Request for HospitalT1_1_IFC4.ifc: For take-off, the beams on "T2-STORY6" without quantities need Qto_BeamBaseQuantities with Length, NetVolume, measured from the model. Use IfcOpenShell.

First a look at what the model holds.

```python
import ifcopenshell
import ifcopenshell.util.element
import ifcopenshell.util.unit

model = ifcopenshell.open("HospitalT1_1_IFC4.ifc")
print(model.schema)
for unit_type in ("LENGTHUNIT", "AREAUNIT", "VOLUMEUNIT"):
    print(unit_type, ifcopenshell.util.unit.calculate_unit_scale(model, unit_type))
storey = next(s for s in model.by_type("IfcBuildingStorey") if s.Name == "T2-STORY6")
beams = [e for e in ifcopenshell.util.element.get_decomposition(storey) if e.is_a("IfcBeam")]
for e in sorted(beams, key=lambda e: e.id()):
    print(e.id(), e.is_a(), e.Name, list(ifcopenshell.util.element.get_psets(e, qtos_only=True)), sep=" | ")
```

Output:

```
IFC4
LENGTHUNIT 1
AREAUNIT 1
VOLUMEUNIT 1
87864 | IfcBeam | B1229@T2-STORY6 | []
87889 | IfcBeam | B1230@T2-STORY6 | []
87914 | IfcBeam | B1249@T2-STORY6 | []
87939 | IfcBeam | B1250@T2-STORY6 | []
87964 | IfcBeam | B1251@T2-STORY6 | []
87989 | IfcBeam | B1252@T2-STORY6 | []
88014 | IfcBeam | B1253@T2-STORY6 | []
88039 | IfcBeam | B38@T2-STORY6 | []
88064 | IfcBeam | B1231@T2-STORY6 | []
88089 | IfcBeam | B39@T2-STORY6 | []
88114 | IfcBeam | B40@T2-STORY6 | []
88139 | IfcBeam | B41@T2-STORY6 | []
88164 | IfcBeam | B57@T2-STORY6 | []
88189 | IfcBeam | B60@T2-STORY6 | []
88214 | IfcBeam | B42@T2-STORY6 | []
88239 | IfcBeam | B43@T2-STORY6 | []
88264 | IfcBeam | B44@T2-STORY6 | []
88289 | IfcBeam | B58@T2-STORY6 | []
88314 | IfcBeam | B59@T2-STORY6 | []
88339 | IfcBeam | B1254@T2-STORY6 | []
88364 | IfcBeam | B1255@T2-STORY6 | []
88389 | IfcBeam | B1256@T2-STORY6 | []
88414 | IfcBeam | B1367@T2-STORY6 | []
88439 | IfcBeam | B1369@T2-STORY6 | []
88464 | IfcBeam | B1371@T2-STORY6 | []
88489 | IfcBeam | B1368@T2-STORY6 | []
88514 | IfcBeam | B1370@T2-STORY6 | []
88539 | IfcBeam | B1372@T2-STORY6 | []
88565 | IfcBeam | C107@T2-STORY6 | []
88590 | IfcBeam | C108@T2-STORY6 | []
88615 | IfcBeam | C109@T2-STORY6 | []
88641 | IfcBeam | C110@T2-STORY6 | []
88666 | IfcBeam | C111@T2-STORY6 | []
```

```python
import ifcopenshell
import ifcopenshell.api.pset
import ifcopenshell.geom
import ifcopenshell.util.element
import ifcopenshell.util.shape
import ifcopenshell.util.unit

model = ifcopenshell.open("HospitalT1_1_IFC4.ifc")
unit_scale = ifcopenshell.util.unit.calculate_unit_scale(model)
volume_scale = ifcopenshell.util.unit.calculate_unit_scale(model, "VOLUMEUNIT")
settings = ifcopenshell.geom.settings()

storey = next(s for s in model.by_type("IfcBuildingStorey") if s.Name == "T2-STORY6")
beams = [e for e in ifcopenshell.util.element.get_decomposition(storey) if e.is_a("IfcBeam")]

for e in sorted(beams, key=lambda e: e.id()):
    if ifcopenshell.util.element.get_psets(e, qtos_only=True, should_inherit=False):
        continue
    # Geometry comes back in metres, in the element's own axes.
    shape = ifcopenshell.geom.create_shape(settings, e)
    values = {
        "Length": ifcopenshell.util.shape.get_max_xyz(shape.geometry) / unit_scale,
        "NetVolume": ifcopenshell.util.shape.get_volume(shape.geometry) / volume_scale,
    }
    qto = ifcopenshell.api.pset.add_qto(model, product=e, name="Qto_BeamBaseQuantities")
    ifcopenshell.api.pset.edit_qto(model, qto=qto, properties=values)
    print(e.id(), {k: round(v, 3) for k, v in values.items()})

model.write("HospitalT1_1_IFC4_v2.ifc")
```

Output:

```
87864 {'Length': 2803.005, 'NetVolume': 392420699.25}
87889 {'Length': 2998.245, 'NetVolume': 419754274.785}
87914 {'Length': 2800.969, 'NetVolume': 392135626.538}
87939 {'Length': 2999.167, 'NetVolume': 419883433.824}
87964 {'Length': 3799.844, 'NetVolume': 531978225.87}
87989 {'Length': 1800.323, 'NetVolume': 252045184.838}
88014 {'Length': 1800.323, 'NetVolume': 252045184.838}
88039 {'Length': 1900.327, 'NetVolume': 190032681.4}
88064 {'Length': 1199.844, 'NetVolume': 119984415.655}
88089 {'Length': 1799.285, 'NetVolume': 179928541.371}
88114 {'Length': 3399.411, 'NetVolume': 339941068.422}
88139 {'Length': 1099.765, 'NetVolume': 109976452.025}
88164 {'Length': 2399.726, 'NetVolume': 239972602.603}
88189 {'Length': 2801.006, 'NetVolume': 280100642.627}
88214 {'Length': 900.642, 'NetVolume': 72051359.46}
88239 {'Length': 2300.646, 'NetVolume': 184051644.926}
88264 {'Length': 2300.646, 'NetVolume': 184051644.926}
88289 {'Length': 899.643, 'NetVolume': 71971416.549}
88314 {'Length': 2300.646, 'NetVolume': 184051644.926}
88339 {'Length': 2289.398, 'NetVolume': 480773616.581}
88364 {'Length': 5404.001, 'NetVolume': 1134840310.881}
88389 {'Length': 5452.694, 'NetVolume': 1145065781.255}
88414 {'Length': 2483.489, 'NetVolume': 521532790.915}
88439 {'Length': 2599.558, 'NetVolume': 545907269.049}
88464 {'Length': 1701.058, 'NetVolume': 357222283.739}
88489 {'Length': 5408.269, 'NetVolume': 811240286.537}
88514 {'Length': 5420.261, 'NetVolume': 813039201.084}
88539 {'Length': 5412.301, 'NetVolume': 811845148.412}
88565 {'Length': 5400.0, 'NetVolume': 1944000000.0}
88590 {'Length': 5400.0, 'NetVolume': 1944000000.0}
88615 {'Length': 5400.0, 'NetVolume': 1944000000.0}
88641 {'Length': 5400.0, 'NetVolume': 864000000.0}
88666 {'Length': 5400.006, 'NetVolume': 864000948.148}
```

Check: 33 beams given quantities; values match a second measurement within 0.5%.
